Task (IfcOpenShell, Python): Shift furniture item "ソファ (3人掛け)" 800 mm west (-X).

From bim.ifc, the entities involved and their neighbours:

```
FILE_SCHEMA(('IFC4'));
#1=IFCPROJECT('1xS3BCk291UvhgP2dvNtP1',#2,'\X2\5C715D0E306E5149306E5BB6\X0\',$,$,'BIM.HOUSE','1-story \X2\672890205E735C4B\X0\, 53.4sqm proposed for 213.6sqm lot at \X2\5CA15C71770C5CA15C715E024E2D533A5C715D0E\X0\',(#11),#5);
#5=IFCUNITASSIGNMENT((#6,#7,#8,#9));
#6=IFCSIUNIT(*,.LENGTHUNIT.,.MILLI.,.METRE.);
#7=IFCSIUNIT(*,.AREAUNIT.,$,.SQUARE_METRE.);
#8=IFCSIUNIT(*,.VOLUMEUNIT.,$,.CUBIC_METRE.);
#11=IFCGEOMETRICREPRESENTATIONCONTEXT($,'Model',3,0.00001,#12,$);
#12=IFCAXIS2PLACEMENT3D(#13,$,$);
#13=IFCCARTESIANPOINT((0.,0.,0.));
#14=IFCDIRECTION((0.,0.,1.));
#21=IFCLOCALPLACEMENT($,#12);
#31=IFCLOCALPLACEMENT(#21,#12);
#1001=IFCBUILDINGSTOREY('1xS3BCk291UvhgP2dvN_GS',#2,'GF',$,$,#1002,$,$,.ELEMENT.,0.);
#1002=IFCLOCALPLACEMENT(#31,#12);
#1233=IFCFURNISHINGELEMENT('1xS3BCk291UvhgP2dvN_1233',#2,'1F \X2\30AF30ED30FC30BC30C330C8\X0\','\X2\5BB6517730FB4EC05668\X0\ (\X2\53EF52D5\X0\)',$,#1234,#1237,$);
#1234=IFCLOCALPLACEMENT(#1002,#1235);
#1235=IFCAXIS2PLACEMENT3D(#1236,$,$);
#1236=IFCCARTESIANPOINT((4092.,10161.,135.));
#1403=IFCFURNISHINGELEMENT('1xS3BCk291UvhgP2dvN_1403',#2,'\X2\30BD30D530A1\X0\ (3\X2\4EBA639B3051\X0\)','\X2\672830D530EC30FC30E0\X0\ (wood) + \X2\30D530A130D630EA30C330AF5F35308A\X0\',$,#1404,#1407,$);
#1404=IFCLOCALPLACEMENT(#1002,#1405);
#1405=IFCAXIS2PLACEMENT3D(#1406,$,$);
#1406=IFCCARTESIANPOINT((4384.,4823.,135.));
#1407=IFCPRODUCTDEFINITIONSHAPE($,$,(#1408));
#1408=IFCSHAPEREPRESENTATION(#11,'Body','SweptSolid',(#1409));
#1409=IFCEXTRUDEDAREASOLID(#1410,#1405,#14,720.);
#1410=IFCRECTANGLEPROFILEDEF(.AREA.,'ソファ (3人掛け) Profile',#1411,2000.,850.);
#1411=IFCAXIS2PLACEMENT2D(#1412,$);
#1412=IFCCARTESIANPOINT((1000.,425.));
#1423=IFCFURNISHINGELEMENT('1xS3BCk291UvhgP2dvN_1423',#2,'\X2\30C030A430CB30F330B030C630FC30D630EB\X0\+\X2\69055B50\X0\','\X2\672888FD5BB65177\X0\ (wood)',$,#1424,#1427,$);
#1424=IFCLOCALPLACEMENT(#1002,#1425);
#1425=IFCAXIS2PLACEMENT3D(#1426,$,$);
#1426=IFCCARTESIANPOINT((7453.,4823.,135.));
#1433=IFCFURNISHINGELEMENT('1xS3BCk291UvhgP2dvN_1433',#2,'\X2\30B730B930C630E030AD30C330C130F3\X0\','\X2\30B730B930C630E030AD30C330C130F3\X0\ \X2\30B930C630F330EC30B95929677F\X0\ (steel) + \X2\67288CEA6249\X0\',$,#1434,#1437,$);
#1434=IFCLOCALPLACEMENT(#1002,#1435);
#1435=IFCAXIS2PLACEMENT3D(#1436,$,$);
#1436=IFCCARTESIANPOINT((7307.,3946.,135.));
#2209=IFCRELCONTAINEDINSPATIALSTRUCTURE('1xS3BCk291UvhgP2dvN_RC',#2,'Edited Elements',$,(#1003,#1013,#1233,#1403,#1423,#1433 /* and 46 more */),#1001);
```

```python
import ifcopenshell
import ifcopenshell.api.geometry
import ifcopenshell.util.placement
import ifcopenshell.util.unit

model = ifcopenshell.open("bim.ifc")
unit_scale = ifcopenshell.util.unit.calculate_unit_scale(model)

item = model.by_id(1403)
matrix = ifcopenshell.util.placement.get_local_placement(item.ObjectPlacement)
matrix[0, 3] -= 0.8 / unit_scale
ifcopenshell.api.geometry.edit_object_placement(model, product=item, matrix=matrix, is_si=False)

print(ifcopenshell.util.placement.get_local_placement(item.ObjectPlacement).round(3) + 0.0)

model.write("bim_updated.ifc")
```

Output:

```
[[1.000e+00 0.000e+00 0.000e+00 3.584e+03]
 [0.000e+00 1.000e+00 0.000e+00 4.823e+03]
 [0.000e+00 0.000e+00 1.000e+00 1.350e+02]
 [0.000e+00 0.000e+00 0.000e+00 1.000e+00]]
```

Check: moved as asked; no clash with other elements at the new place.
